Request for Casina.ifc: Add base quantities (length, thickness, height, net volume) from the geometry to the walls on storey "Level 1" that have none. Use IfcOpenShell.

First a look at what the model holds.

```python
import ifcopenshell
import ifcopenshell.util.element
import ifcopenshell.util.unit

model = ifcopenshell.open("Casina.ifc")
print(model.schema)
for unit_type in ("LENGTHUNIT", "AREAUNIT", "VOLUMEUNIT"):
    print(unit_type, ifcopenshell.util.unit.calculate_unit_scale(model, unit_type))
storey = next(s for s in model.by_type("IfcBuildingStorey") if s.Name == "Level 1")
walls = [e for e in ifcopenshell.util.element.get_decomposition(storey) if e.is_a("IfcWall")]
for e in sorted(walls, key=lambda e: e.id()):
    print(e.id(), e.is_a(), e.Name, list(ifcopenshell.util.element.get_psets(e, qtos_only=True)), sep=" | ")
```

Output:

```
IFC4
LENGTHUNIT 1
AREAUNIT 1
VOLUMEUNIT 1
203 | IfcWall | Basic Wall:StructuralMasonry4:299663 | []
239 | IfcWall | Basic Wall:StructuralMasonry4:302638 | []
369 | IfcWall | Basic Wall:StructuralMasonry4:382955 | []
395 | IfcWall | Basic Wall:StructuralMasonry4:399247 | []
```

```python
import ifcopenshell
import ifcopenshell.api.pset
import ifcopenshell.geom
import ifcopenshell.util.element
import ifcopenshell.util.shape
import ifcopenshell.util.unit

model = ifcopenshell.open("Casina.ifc")
unit_scale = ifcopenshell.util.unit.calculate_unit_scale(model)
volume_scale = ifcopenshell.util.unit.calculate_unit_scale(model, "VOLUMEUNIT")
settings = ifcopenshell.geom.settings()

storey = next(s for s in model.by_type("IfcBuildingStorey") if s.Name == "Level 1")
walls = [e for e in ifcopenshell.util.element.get_decomposition(storey) if e.is_a("IfcWall")]

for e in sorted(walls, key=lambda e: e.id()):
    if ifcopenshell.util.element.get_psets(e, qtos_only=True, should_inherit=False):
        continue
    # Geometry comes back in metres, in the element's own axes.
    shape = ifcopenshell.geom.create_shape(settings, e)
    values = {
        "Length": ifcopenshell.util.shape.get_x(shape.geometry) / unit_scale,
        "Width": ifcopenshell.util.shape.get_y(shape.geometry) / unit_scale,
        "Height": ifcopenshell.util.shape.get_z(shape.geometry) / unit_scale,
        "NetVolume": ifcopenshell.util.shape.get_volume(shape.geometry) / volume_scale,
    }
    qto = ifcopenshell.api.pset.add_qto(model, product=e, name="Qto_WallBaseQuantities")
    ifcopenshell.api.pset.edit_qto(model, qto=qto, properties=values)
    print(e.id(), {k: round(v, 3) for k, v in values.items()})

model.write("Casina_updated.ifc")
```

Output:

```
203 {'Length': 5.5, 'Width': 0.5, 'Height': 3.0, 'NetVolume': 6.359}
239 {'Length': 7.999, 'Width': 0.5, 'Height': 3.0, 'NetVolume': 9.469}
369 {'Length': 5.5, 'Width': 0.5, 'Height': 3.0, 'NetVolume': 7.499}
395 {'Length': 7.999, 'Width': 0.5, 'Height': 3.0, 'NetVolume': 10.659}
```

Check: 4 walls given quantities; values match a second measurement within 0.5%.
